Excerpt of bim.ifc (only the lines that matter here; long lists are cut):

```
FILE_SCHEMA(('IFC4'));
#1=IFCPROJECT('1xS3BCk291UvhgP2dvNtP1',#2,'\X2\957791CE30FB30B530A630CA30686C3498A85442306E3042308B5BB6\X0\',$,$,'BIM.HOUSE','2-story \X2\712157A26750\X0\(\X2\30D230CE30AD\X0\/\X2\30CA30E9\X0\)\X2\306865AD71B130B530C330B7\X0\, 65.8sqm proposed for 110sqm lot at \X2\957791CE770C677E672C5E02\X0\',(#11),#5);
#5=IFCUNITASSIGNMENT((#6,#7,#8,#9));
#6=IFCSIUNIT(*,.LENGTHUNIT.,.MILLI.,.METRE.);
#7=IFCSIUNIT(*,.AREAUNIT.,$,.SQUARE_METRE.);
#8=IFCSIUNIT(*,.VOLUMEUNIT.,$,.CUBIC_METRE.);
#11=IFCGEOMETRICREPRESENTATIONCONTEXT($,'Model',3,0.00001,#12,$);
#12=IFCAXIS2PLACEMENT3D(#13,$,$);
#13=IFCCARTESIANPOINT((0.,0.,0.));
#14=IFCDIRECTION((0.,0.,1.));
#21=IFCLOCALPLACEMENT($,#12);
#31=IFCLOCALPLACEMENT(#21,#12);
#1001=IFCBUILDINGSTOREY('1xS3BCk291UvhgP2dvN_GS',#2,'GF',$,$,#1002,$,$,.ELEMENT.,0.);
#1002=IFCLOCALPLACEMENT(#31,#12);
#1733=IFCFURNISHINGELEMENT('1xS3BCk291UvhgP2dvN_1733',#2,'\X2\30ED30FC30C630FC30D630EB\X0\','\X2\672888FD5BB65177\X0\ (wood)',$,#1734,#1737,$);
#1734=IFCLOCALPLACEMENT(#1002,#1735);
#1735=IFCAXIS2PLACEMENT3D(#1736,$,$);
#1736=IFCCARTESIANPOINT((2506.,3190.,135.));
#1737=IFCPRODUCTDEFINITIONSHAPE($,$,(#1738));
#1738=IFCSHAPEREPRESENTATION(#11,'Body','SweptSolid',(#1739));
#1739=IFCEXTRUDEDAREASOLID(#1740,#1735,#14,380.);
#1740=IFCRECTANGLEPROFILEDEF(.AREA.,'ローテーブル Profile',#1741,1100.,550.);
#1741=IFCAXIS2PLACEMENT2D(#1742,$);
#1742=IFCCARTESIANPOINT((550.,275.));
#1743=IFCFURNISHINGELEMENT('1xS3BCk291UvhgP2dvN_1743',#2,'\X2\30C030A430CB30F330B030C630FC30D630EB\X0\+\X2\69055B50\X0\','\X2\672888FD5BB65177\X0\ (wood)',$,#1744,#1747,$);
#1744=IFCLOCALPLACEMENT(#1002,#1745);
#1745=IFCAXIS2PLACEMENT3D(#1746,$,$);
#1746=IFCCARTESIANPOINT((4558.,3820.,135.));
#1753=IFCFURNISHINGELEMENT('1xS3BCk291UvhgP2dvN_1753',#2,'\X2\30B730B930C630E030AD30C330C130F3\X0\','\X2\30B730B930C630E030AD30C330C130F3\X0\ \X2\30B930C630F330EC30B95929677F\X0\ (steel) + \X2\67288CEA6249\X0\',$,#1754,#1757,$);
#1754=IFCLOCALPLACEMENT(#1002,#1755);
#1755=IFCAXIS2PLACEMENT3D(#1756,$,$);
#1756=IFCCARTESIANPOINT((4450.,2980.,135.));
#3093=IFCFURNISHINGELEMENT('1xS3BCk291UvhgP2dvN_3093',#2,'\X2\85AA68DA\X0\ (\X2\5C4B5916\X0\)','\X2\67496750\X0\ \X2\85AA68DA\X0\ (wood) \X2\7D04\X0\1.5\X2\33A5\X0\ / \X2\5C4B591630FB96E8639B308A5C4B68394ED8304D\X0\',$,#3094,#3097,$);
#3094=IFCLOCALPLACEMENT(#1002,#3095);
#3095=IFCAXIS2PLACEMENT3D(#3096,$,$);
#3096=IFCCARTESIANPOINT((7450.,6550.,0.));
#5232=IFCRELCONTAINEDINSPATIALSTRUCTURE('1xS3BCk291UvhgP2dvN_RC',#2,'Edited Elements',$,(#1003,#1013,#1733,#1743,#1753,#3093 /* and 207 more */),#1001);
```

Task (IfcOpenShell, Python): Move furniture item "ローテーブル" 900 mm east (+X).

```python
import ifcopenshell
import ifcopenshell.api.geometry
import ifcopenshell.util.placement

model = ifcopenshell.open("bim.ifc")

item = model.by_guid("1xS3BCk291UvhgP2dvN_1733")
matrix = ifcopenshell.util.placement.get_local_placement(item.ObjectPlacement)
matrix[0, 3] += 900.0
ifcopenshell.api.geometry.edit_object_placement(model, product=item, matrix=matrix, is_si=False)

print(ifcopenshell.util.placement.get_local_placement(item.ObjectPlacement).round(3) + 0.0)

model.write("bim_updated.ifc")
```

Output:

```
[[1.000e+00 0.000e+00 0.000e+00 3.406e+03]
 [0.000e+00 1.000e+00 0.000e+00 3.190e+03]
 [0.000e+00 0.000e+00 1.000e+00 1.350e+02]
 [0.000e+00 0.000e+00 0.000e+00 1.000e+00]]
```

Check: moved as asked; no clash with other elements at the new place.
